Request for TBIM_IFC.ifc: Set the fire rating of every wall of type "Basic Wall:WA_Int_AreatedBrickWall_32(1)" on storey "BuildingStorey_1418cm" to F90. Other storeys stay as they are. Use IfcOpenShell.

First a look at what the model holds.

```python
import ifcopenshell
import ifcopenshell.util.element

model = ifcopenshell.open("TBIM_IFC.ifc")
print(model.schema)
storey = next(s for s in model.by_type("IfcBuildingStorey") if s.Name == "BuildingStorey_1418cm")
walls = [e for e in ifcopenshell.util.element.get_decomposition(storey) if e.is_a("IfcWall")]
seen = {}
for e in walls:
    element_type = ifcopenshell.util.element.get_type(e)
    key = (element_type.Name if element_type != e and element_type else None, ifcopenshell.util.element.get_pset(e, "Pset_WallCommon", "FireRating"))
    seen[key] = seen.get(key, 0) + 1
for (name, value), count in sorted(seen.items(), key=str):
    print(count, "x", name, "|", value)
```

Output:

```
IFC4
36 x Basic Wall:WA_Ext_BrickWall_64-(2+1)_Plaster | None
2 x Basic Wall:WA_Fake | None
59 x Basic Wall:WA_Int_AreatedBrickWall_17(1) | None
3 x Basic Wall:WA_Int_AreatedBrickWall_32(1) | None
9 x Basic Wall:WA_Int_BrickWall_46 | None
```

```python
import ifcopenshell
import ifcopenshell.api.pset
import ifcopenshell.util.element

model = ifcopenshell.open("TBIM_IFC.ifc")

storey = next(s for s in model.by_type("IfcBuildingStorey") if s.Name == "BuildingStorey_1418cm")
walls = [e for e in ifcopenshell.util.element.get_decomposition(storey) if e.is_a("IfcWall")]

count = 0
for e in walls:
    element_type = ifcopenshell.util.element.get_type(e)
    if element_type in (None, e) or element_type.Name != "Basic Wall:WA_Int_AreatedBrickWall_32(1)":
        continue
    # add_pset returns the element's existing set when there is one.
    pset = ifcopenshell.api.pset.add_pset(model, product=e, name="Pset_WallCommon")
    ifcopenshell.api.pset.edit_pset(model, pset=pset, properties={"FireRating": "F90"})
    count += 1

print(count, "walls updated")

model.write("TBIM_IFC_v2.ifc")
```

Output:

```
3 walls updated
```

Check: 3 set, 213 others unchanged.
